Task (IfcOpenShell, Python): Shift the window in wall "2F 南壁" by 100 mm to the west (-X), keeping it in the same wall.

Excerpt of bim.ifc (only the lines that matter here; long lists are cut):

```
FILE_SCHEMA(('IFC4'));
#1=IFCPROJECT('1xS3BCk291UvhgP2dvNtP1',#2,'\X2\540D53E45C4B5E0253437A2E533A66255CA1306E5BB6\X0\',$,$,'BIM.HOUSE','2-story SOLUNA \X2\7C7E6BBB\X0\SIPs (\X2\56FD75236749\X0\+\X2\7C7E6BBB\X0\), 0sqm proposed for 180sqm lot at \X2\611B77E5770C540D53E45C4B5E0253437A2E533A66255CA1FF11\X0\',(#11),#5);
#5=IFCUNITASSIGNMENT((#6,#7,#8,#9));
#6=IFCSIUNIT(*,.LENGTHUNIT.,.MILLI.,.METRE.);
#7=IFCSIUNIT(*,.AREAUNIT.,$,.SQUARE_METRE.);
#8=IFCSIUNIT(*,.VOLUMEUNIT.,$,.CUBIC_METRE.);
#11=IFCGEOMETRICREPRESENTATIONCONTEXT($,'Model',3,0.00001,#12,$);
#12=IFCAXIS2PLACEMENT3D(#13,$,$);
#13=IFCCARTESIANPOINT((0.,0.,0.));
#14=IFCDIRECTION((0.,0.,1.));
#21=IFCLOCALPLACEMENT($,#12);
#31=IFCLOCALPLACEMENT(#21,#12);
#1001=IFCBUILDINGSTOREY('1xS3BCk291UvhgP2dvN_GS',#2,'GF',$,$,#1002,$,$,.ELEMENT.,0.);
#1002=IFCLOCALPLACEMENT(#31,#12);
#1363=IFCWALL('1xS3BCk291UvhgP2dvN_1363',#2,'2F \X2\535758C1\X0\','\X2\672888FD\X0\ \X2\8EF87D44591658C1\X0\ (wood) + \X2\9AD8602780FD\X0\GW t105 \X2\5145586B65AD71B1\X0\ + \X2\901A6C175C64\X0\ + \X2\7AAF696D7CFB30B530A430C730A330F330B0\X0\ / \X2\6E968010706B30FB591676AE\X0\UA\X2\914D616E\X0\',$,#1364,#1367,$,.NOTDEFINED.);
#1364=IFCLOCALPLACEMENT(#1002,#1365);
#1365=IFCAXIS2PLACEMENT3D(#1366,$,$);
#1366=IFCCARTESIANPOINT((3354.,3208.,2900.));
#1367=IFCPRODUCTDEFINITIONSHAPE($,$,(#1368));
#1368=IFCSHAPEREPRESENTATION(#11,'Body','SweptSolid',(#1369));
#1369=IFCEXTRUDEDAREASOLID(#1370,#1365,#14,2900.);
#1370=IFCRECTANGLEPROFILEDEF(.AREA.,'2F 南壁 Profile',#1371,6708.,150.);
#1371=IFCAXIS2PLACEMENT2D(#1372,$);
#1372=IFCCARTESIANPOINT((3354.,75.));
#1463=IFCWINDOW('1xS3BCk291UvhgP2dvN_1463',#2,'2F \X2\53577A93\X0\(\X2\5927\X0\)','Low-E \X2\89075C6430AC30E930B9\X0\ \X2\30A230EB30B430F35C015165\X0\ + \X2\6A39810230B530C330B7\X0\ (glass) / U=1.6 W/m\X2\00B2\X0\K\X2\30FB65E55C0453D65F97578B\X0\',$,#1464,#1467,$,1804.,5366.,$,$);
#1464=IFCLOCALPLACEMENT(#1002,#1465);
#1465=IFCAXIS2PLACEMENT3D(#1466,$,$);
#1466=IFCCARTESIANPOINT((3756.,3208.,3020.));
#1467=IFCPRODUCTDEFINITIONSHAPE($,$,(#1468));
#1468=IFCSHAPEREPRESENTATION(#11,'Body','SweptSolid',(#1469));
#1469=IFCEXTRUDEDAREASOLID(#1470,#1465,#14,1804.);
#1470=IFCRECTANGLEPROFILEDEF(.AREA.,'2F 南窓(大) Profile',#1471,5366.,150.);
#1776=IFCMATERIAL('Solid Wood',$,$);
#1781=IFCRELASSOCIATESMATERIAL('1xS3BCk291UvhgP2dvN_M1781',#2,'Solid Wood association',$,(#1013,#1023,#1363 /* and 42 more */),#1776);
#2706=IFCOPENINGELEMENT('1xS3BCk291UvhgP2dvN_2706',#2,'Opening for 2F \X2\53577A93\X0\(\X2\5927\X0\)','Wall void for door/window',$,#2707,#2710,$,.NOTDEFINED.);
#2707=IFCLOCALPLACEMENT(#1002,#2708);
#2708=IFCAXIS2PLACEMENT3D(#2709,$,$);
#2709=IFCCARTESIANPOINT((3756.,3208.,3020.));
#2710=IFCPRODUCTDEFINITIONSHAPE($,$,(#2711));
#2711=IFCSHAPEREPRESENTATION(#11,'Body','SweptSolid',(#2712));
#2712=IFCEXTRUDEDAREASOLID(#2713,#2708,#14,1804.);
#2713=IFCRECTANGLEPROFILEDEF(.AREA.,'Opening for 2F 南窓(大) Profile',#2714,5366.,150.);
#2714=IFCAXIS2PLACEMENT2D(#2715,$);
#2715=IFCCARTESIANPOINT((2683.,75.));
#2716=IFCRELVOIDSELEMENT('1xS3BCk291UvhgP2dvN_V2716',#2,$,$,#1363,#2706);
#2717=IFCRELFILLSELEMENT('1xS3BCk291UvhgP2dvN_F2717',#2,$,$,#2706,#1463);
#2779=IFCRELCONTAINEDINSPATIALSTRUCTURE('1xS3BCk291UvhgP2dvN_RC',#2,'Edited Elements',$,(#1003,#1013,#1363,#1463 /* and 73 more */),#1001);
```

```python
import ifcopenshell
import ifcopenshell.api.geometry
import ifcopenshell.util.placement
import ifcopenshell.util.unit

model = ifcopenshell.open("bim.ifc")
unit_scale = ifcopenshell.util.unit.calculate_unit_scale(model)

window = model.by_guid("1xS3BCk291UvhgP2dvN_1463")
opening = window.FillsVoids[0].RelatingOpeningElement
wall = opening.VoidsElements[0].RelatingBuildingElement

wall_matrix = ifcopenshell.util.placement.get_local_placement(wall.ObjectPlacement)
shift = wall_matrix[:3, 0] * -0.1 / unit_scale
before = ifcopenshell.util.placement.get_local_placement(window.ObjectPlacement)[:3, 3].copy()

# The window is not placed relative to its opening, so move both.
for product in (opening, window):
    matrix = ifcopenshell.util.placement.get_local_placement(product.ObjectPlacement)
    matrix[:3, 3] += shift
    ifcopenshell.api.geometry.edit_object_placement(model, product=product, matrix=matrix, is_si=False)

after = ifcopenshell.util.placement.get_local_placement(window.ObjectPlacement)[:3, 3]
print("window moved by", (after - before).round(3) + 0.0)

model.write("bim_edited.ifc")
```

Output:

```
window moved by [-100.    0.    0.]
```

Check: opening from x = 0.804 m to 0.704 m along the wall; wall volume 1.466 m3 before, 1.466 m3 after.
